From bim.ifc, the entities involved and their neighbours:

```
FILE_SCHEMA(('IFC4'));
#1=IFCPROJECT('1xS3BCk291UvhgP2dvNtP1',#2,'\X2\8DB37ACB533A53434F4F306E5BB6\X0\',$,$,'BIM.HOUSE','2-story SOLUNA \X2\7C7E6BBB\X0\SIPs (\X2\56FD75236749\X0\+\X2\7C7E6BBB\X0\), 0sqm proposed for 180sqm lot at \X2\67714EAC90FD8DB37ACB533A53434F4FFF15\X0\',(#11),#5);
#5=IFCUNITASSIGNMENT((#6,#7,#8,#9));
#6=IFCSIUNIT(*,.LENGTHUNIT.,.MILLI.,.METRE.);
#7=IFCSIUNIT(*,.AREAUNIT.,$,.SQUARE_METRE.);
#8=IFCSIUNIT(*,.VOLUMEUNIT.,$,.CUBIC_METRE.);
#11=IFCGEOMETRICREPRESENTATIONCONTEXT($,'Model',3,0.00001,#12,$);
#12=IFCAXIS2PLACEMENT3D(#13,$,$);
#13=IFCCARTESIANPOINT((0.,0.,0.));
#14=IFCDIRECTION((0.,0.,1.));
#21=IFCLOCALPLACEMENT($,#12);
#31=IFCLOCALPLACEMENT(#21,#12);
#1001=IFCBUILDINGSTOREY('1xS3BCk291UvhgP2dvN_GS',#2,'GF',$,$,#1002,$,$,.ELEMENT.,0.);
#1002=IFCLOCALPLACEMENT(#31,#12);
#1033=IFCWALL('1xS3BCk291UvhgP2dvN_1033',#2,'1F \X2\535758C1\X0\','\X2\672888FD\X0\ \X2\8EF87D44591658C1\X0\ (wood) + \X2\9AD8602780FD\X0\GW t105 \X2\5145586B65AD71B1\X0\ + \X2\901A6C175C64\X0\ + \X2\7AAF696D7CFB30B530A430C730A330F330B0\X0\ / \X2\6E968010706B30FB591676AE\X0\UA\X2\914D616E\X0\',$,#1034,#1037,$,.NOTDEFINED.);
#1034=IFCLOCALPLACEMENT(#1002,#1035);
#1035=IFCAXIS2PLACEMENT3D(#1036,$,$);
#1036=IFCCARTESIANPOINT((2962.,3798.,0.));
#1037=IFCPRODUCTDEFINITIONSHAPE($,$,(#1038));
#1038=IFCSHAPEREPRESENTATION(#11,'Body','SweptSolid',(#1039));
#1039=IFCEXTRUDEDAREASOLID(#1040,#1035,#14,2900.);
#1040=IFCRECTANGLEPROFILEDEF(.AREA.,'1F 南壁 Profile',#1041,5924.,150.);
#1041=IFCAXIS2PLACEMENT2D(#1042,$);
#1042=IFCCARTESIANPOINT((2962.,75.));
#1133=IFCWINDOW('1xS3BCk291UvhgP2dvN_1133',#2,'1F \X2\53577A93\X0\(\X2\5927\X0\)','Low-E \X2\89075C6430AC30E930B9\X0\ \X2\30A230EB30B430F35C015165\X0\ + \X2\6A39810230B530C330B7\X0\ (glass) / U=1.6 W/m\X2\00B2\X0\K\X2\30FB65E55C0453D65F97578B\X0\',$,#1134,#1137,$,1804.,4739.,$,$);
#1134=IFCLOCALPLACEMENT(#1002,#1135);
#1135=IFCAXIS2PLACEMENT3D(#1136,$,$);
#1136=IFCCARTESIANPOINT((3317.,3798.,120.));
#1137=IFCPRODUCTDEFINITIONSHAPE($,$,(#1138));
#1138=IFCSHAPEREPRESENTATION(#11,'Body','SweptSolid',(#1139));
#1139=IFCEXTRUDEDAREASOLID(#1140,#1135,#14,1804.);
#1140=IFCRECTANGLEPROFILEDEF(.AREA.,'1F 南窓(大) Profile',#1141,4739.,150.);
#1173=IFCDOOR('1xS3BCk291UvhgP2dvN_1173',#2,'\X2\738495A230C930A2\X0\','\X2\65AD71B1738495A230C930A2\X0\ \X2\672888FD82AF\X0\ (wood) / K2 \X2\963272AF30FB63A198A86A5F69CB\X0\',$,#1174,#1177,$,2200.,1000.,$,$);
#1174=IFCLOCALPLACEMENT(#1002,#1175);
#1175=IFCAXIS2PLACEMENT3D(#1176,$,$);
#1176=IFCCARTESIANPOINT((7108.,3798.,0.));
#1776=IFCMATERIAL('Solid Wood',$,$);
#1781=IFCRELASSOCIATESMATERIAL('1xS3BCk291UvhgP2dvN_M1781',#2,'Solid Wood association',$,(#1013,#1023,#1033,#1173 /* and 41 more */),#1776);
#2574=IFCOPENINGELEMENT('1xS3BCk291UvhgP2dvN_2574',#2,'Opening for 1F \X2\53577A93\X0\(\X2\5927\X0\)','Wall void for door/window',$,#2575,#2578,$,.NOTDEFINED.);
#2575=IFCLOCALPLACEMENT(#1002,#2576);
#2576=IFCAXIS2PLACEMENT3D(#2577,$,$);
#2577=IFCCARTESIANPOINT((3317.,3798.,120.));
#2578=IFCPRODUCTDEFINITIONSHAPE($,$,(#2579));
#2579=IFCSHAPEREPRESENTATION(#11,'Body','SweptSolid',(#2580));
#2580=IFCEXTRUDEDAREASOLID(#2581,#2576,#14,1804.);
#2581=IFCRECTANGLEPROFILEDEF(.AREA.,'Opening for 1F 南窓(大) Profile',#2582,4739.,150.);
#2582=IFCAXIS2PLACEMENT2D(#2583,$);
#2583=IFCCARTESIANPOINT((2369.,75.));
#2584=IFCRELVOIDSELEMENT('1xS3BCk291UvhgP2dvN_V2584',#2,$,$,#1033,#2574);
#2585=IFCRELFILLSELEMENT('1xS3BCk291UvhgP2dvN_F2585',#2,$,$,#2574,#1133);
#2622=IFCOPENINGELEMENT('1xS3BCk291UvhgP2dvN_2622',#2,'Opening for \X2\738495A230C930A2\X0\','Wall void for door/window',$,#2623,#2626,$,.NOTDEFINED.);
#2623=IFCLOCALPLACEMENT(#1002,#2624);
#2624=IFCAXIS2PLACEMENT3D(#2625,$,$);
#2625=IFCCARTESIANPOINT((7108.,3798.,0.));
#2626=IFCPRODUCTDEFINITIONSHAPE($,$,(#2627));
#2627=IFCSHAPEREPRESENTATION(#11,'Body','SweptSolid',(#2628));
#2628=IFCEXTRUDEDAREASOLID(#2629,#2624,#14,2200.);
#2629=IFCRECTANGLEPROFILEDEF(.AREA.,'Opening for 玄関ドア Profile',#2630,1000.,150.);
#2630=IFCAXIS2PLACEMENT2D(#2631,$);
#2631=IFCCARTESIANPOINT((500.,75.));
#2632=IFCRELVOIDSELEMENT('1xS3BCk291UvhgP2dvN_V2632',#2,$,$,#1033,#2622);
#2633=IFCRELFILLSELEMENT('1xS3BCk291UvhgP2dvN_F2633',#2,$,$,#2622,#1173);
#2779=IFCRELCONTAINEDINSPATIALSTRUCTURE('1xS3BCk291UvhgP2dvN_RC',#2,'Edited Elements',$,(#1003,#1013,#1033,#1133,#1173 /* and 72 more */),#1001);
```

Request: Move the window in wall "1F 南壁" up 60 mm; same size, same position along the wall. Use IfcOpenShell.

```python
import numpy as np
import ifcopenshell
import ifcopenshell.api.geometry
import ifcopenshell.util.placement
import ifcopenshell.util.unit

model = ifcopenshell.open("bim.ifc")
unit_scale = ifcopenshell.util.unit.calculate_unit_scale(model)

window = model.by_guid("1xS3BCk291UvhgP2dvN_1133")
opening = window.FillsVoids[0].RelatingOpeningElement
dz = 60.0

shift = np.array([0.0, 0.0, dz])
# The window is not placed relative to its opening, so move both.
for product in (opening, window):
    matrix = ifcopenshell.util.placement.get_local_placement(product.ObjectPlacement)
    matrix[:3, 3] += shift
    ifcopenshell.api.geometry.edit_object_placement(model, product=product, matrix=matrix, is_si=False)

print(f"moved by {dz * unit_scale:+.3f} m")

model.write("bim-out.ifc")
```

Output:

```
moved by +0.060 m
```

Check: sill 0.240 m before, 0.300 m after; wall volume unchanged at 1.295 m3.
